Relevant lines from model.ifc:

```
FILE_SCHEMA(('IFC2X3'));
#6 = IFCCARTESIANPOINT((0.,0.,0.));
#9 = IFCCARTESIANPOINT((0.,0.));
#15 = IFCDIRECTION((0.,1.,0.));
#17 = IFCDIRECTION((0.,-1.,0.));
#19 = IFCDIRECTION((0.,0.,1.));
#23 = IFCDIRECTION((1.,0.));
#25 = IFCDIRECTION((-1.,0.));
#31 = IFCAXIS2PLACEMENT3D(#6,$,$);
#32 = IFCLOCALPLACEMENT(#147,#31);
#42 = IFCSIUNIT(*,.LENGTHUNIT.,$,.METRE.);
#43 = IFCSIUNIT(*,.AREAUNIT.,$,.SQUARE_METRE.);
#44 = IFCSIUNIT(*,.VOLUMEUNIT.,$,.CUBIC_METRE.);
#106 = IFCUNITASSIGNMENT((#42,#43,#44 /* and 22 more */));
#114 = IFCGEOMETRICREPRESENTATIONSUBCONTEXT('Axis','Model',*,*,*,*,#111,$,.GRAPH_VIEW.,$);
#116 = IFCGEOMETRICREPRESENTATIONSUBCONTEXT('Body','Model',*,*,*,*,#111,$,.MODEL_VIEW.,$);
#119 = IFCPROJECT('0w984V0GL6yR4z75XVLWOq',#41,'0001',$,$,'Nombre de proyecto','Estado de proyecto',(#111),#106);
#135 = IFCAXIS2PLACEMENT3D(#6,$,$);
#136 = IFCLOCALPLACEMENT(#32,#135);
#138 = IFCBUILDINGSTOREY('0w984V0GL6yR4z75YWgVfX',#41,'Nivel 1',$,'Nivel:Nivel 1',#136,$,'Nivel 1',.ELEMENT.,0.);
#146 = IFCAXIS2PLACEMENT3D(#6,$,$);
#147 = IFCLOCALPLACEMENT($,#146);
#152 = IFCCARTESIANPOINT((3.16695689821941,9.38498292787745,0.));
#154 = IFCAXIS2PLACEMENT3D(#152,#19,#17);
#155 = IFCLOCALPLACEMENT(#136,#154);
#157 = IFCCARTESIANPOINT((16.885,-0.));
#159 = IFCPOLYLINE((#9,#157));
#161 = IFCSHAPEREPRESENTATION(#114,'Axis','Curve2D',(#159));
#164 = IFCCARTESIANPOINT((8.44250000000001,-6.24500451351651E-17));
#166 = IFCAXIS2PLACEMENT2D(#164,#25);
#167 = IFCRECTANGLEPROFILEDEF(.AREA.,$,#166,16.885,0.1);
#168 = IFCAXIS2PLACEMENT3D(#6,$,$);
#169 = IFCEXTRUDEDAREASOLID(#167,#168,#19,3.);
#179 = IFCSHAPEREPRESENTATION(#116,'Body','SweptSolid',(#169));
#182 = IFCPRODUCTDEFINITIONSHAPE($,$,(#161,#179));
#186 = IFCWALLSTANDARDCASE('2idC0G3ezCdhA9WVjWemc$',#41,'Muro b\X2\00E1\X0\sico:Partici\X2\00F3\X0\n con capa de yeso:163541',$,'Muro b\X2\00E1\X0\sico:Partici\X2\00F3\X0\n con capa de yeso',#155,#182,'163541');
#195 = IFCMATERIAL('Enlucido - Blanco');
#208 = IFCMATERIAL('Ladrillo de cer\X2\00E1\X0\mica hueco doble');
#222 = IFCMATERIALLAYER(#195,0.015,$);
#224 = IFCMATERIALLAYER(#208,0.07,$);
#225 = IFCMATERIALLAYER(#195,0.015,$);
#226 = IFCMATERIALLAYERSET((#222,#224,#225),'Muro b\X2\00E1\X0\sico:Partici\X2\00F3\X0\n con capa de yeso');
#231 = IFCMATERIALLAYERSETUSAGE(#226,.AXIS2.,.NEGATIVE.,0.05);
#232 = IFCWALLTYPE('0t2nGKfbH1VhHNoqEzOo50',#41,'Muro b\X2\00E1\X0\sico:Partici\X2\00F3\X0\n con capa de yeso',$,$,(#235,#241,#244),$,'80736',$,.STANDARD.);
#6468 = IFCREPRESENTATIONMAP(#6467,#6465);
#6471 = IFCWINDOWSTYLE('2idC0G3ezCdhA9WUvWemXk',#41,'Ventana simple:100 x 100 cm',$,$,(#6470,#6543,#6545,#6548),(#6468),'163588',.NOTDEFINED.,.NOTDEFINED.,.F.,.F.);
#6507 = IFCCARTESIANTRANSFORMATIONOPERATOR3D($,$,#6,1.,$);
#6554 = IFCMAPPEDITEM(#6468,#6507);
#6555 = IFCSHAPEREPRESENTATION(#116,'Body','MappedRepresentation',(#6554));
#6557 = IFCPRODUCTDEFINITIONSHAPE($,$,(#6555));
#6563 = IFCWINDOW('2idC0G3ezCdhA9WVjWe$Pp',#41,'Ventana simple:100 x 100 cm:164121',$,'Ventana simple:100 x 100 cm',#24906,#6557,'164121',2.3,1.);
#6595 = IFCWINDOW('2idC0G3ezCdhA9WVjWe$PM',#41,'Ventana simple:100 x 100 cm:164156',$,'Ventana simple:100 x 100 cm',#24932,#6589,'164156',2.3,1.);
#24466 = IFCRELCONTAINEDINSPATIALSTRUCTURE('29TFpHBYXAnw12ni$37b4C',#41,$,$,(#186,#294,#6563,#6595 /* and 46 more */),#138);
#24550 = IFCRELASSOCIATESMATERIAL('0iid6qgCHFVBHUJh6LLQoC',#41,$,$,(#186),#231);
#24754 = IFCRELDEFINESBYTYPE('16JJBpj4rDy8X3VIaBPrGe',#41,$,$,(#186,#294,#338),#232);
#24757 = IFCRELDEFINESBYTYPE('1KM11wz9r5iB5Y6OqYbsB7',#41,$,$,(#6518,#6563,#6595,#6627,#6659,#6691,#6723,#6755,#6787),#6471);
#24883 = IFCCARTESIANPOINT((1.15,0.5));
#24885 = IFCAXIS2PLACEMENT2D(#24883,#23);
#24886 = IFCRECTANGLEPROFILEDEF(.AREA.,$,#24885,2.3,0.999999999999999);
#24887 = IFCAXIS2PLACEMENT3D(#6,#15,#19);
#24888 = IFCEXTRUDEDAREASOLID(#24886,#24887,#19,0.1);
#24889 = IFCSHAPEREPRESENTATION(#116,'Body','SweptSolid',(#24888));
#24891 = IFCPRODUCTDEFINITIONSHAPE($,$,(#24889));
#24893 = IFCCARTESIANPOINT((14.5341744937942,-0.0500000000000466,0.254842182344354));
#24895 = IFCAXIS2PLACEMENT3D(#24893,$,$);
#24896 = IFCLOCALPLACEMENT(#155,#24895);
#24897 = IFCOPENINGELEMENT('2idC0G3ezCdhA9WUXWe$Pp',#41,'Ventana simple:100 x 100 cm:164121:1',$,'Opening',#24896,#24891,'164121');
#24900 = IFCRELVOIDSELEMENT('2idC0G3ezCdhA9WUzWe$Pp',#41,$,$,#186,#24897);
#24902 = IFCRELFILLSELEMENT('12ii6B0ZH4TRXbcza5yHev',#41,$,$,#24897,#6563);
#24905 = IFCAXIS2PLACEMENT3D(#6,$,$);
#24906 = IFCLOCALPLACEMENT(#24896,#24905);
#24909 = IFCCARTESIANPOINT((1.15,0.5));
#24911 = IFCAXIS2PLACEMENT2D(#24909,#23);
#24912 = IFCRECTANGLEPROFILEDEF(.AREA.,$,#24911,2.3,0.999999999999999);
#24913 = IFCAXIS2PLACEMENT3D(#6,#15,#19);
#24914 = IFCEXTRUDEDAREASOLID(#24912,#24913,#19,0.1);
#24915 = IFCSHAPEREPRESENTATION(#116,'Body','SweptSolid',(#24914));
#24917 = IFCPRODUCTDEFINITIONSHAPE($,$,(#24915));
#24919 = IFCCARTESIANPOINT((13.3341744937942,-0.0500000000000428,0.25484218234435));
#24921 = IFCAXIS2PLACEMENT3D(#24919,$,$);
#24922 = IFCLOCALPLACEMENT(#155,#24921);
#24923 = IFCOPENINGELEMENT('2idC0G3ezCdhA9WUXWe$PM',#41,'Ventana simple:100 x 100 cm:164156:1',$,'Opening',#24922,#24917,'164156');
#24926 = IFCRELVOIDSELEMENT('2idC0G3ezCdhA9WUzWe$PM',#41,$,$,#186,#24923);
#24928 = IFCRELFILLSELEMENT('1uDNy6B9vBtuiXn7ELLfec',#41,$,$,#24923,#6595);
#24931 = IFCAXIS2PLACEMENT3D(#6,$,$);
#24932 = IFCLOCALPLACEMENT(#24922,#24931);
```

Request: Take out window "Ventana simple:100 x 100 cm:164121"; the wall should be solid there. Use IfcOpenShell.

```python
import ifcopenshell
import ifcopenshell.api.feature
import ifcopenshell.api.root
import ifcopenshell.geom
import ifcopenshell.util.shape

model = ifcopenshell.open("model.ifc")
settings = ifcopenshell.geom.settings()


def volume(element):
    """Net volume in cubic metres, openings subtracted."""
    shape = ifcopenshell.geom.create_shape(settings, element)
    return ifcopenshell.util.shape.get_volume(shape.geometry)


window = model.by_guid("2idC0G3ezCdhA9WVjWe$Pp")
opening = window.FillsVoids[0].RelatingOpeningElement
wall = opening.VoidsElements[0].RelatingBuildingElement
before = volume(wall)

ifcopenshell.api.root.remove_product(model, product=window)
ifcopenshell.api.feature.remove_feature(model, feature=opening)

after = volume(wall)

print(f"wall volume {before:.3f} -> {after:.3f} m3")

model.write("model_v2.ifc")
```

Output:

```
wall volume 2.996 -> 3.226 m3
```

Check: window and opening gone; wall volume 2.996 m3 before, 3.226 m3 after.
